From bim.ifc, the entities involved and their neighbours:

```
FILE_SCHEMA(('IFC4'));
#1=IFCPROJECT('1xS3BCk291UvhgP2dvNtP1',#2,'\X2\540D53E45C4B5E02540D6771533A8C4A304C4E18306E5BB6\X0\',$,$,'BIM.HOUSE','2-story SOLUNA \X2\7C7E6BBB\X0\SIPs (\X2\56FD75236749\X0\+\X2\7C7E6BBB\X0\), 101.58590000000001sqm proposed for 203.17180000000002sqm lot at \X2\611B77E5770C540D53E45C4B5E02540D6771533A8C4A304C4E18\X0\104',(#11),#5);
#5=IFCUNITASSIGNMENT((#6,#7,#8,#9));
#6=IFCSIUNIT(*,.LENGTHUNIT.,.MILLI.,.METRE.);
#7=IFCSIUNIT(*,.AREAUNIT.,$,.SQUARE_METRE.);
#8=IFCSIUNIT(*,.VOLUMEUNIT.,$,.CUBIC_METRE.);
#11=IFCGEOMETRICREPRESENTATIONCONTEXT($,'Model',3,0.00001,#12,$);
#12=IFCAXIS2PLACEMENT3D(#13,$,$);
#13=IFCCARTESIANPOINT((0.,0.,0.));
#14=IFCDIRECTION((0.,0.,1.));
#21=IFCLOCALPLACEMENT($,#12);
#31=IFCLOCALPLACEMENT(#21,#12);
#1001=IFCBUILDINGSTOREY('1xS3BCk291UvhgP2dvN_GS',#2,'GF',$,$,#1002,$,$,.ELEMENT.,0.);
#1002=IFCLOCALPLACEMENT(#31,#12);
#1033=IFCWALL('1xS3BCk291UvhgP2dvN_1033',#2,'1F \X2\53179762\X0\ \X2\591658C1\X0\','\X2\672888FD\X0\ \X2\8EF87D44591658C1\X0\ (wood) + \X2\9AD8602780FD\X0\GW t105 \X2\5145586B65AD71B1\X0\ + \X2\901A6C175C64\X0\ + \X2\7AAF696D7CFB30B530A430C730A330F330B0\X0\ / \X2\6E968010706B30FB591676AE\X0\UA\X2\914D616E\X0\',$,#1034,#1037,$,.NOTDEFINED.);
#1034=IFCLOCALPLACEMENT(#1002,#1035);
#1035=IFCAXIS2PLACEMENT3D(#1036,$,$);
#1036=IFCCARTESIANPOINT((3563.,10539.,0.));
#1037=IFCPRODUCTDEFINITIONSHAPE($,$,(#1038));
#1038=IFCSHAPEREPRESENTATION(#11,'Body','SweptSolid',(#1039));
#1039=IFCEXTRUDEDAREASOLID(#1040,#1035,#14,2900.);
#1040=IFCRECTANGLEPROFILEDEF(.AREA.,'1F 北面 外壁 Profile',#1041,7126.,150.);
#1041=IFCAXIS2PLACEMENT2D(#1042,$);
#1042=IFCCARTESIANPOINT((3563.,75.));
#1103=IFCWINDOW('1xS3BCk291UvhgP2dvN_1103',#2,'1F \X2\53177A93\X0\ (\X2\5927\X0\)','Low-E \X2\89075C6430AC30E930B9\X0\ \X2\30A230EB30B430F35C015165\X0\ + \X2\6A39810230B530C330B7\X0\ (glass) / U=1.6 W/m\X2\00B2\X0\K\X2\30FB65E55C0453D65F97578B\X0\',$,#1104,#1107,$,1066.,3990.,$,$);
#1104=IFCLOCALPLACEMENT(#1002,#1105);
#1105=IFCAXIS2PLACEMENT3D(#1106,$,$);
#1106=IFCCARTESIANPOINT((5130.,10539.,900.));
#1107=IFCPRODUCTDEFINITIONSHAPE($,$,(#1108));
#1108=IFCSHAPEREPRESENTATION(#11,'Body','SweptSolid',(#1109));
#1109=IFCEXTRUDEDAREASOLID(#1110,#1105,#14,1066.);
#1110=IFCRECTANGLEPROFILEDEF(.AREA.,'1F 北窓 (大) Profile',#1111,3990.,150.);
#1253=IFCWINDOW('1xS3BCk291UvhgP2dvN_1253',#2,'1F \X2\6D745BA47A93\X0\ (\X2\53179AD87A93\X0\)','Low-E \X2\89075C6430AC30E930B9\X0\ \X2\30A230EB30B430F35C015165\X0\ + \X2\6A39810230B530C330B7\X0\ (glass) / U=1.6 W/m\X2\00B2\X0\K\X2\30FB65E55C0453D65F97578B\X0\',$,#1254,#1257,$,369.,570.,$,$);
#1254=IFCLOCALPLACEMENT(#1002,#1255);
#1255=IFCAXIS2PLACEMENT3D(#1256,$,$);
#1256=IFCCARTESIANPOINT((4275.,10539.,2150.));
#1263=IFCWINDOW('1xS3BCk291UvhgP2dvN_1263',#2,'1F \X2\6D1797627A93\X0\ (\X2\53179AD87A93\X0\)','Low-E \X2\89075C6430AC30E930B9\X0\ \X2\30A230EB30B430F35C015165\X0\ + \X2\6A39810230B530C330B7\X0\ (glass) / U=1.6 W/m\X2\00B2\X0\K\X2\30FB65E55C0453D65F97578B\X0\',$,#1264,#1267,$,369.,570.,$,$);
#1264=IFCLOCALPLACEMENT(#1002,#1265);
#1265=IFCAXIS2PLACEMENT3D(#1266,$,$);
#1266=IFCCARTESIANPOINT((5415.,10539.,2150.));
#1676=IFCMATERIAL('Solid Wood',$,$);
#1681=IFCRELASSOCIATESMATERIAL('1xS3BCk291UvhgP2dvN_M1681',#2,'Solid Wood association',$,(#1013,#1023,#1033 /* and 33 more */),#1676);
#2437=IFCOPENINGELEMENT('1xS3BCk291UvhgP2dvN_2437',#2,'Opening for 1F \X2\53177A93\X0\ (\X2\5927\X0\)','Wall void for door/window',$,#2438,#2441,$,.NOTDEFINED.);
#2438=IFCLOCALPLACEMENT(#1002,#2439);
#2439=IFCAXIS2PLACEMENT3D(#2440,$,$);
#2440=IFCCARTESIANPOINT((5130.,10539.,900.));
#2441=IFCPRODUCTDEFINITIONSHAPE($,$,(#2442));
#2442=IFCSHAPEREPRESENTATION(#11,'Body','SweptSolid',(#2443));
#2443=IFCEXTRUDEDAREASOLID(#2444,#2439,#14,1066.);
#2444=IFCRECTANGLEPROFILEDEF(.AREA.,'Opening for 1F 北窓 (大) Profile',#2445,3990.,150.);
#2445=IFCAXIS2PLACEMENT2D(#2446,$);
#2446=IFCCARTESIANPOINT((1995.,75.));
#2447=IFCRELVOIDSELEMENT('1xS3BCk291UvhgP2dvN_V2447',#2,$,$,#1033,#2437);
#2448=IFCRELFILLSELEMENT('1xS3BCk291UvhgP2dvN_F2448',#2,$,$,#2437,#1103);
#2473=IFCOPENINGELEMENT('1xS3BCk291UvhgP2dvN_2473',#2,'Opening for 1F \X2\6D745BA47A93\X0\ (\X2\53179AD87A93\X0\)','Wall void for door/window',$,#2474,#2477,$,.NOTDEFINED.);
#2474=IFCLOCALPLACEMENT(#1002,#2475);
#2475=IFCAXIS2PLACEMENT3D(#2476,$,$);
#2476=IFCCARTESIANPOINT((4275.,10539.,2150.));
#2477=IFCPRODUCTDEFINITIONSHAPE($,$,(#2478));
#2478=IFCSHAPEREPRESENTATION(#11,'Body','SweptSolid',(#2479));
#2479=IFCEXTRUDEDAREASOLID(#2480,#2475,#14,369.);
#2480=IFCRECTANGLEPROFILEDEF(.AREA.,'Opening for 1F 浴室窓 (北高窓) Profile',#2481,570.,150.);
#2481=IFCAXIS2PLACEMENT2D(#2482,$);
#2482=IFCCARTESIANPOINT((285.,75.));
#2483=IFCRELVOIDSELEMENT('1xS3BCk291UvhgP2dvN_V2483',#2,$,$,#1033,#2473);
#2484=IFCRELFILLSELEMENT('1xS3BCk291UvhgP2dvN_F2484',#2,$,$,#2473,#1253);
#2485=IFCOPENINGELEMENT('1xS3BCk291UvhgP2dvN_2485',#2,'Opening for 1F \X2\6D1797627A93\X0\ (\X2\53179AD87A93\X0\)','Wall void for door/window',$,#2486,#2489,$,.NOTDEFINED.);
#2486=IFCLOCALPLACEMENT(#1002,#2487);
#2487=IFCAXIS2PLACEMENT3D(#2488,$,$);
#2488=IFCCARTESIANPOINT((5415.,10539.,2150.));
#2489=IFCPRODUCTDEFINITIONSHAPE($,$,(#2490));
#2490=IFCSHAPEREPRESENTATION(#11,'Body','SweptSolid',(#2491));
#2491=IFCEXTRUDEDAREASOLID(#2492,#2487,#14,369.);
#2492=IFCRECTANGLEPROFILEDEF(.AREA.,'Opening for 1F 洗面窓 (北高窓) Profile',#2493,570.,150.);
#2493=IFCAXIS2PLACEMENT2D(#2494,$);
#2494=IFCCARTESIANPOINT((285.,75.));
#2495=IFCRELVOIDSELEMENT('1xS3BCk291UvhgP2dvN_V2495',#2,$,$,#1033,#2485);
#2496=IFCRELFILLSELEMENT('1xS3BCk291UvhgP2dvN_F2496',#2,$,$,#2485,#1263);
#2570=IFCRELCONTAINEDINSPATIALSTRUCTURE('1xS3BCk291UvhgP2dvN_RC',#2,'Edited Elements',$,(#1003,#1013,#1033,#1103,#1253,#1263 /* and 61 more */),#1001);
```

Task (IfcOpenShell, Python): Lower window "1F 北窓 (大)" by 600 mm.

```python
import numpy as np
import ifcopenshell
import ifcopenshell.api.geometry
import ifcopenshell.util.placement
import ifcopenshell.util.unit

model = ifcopenshell.open("bim.ifc")
unit_scale = ifcopenshell.util.unit.calculate_unit_scale(model)

window = model.by_id(1103)
opening = window.FillsVoids[0].RelatingOpeningElement
dz = -0.6 / unit_scale

shift = np.array([0.0, 0.0, dz])
# The window is not placed relative to its opening, so move both.
for product in (opening, window):
    matrix = ifcopenshell.util.placement.get_local_placement(product.ObjectPlacement)
    matrix[:3, 3] += shift
    ifcopenshell.api.geometry.edit_object_placement(model, product=product, matrix=matrix, is_si=False)

print(f"moved by {dz * unit_scale:+.3f} m")

model.write("bim-out.ifc")
```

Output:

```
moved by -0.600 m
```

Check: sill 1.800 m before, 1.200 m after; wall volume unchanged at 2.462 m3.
